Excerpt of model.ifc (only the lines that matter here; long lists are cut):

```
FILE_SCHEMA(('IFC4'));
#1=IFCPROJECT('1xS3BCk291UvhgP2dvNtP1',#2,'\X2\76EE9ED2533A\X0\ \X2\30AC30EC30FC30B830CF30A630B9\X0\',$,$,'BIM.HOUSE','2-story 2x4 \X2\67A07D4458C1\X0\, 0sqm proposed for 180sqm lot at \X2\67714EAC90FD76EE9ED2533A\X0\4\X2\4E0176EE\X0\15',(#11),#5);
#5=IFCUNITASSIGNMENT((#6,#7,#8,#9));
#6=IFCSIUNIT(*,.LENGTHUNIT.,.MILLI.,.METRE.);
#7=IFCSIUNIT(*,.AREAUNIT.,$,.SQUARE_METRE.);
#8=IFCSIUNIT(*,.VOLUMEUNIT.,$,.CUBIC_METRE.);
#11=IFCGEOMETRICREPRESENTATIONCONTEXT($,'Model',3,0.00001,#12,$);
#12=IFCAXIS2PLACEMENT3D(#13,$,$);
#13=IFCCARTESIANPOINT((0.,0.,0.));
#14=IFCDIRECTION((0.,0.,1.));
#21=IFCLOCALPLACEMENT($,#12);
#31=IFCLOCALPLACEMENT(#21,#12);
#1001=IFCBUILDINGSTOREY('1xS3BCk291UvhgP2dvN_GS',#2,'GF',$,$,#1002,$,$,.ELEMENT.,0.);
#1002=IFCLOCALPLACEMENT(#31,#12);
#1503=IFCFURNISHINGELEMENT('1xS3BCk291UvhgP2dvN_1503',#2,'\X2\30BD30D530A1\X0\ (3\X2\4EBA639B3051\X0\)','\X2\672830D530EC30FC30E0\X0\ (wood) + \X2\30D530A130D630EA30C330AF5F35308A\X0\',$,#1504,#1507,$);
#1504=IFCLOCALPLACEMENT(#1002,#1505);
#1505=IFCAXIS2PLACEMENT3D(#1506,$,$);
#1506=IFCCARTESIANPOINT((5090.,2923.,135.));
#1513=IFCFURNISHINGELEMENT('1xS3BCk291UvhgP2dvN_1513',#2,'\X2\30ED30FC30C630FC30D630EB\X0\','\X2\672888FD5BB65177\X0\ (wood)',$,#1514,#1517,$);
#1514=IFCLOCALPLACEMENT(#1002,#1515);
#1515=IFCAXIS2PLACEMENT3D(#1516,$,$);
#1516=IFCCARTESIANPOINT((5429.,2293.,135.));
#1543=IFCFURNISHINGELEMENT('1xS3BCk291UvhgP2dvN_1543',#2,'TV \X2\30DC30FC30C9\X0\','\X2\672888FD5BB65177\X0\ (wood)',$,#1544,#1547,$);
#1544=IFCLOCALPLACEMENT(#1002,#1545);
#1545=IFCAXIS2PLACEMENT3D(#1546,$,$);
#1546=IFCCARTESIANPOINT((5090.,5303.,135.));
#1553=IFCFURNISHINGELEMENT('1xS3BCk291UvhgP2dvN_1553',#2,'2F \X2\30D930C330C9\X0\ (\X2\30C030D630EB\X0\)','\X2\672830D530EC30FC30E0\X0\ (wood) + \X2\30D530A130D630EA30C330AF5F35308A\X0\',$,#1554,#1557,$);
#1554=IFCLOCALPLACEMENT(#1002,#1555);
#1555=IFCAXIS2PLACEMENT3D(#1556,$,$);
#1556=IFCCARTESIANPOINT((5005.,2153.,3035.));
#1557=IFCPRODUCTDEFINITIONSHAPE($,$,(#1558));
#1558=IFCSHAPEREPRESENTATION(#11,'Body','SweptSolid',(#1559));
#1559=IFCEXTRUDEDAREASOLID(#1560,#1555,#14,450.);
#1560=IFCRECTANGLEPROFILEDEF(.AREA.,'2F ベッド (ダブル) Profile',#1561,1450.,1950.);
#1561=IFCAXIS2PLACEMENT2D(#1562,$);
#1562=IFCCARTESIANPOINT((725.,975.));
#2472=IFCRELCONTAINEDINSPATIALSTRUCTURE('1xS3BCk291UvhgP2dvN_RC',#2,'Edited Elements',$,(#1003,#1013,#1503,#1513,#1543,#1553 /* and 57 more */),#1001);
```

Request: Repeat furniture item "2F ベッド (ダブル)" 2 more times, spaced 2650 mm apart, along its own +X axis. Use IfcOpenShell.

```python
import ifcopenshell
import ifcopenshell.api.geometry
import ifcopenshell.api.root
import ifcopenshell.util.element
import ifcopenshell.util.placement
import ifcopenshell.util.unit

model = ifcopenshell.open("model.ifc")
unit_scale = ifcopenshell.util.unit.calculate_unit_scale(model)


def reuse_history(source, copy):
    """copy_class also copies each property set's owner history, people and application; keep the originals."""
    for rel in copy.IsDefinedBy:
        if rel.is_a("IfcRelDefinesByProperties") and (history := rel.RelatingPropertyDefinition.OwnerHistory):
            rel.RelatingPropertyDefinition.OwnerHistory = source.OwnerHistory
            ifcopenshell.util.element.remove_deep2(model, history)


source = model.by_id(1553)
base = ifcopenshell.util.placement.get_local_placement(source.ObjectPlacement)
step = base[:3, 0] * 2.65 / unit_scale

for i in range(1, 3):
    copy = ifcopenshell.api.root.copy_class(model, product=source)
    copy.Representation = ifcopenshell.util.element.copy_deep(
        model, source.Representation, exclude=["IfcGeometricRepresentationContext", "IfcRepresentationMap"]
    )
    reuse_history(source, copy)
    matrix = base.copy()
    matrix[:3, 3] += i * step
    print("added at", matrix[:3, 3].round(3) + 0.0)
    ifcopenshell.api.geometry.edit_object_placement(model, product=copy, matrix=matrix, is_si=False)

model.write("model_v2.ifc")
```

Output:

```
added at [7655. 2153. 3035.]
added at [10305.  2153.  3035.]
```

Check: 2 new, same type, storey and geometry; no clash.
